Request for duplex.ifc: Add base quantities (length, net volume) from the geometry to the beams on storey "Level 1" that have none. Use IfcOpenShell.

First a look at what the model holds.

```python
import ifcopenshell
import ifcopenshell.util.element
import ifcopenshell.util.unit

model = ifcopenshell.open("duplex.ifc")
print(model.schema)
for unit_type in ("LENGTHUNIT", "AREAUNIT", "VOLUMEUNIT"):
    print(unit_type, ifcopenshell.util.unit.calculate_unit_scale(model, unit_type))
storey = next(s for s in model.by_type("IfcBuildingStorey") if s.Name == "Level 1")
beams = [e for e in ifcopenshell.util.element.get_decomposition(storey) if e.is_a("IfcBeam")]
for e in sorted(beams, key=lambda e: e.id()):
    print(e.id(), e.is_a(), e.Name, list(ifcopenshell.util.element.get_psets(e, qtos_only=True)), sep=" | ")
```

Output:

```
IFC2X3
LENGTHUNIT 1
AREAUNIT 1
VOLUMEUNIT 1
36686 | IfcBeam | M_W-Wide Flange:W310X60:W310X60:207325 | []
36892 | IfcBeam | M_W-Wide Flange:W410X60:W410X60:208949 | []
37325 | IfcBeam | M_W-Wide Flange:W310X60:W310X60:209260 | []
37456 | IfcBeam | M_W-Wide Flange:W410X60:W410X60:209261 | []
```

```python
import ifcopenshell
import ifcopenshell.api.pset
import ifcopenshell.geom
import ifcopenshell.util.element
import ifcopenshell.util.shape
import ifcopenshell.util.unit

model = ifcopenshell.open("duplex.ifc")
unit_scale = ifcopenshell.util.unit.calculate_unit_scale(model)
volume_scale = ifcopenshell.util.unit.calculate_unit_scale(model, "VOLUMEUNIT")
settings = ifcopenshell.geom.settings()

storey = next(s for s in model.by_type("IfcBuildingStorey") if s.Name == "Level 1")
beams = [e for e in ifcopenshell.util.element.get_decomposition(storey) if e.is_a("IfcBeam")]

for e in sorted(beams, key=lambda e: e.id()):
    if ifcopenshell.util.element.get_psets(e, qtos_only=True, should_inherit=False):
        continue
    # Geometry comes back in metres, in the element's own axes.
    shape = ifcopenshell.geom.create_shape(settings, e)
    values = {
        "Length": ifcopenshell.util.shape.get_max_xyz(shape.geometry) / unit_scale,
        "NetVolume": ifcopenshell.util.shape.get_volume(shape.geometry) / volume_scale,
    }
    qto = ifcopenshell.api.pset.add_qto(model, product=e, name="BaseQuantities")
    ifcopenshell.api.pset.edit_qto(model, qto=qto, properties=values)
    print(e.id(), {k: round(v, 3) for k, v in values.items()})

model.write("duplex_rev.ifc")
```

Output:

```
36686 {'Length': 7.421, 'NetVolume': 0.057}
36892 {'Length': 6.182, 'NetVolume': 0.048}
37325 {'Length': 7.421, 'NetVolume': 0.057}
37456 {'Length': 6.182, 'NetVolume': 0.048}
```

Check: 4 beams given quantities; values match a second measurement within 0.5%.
